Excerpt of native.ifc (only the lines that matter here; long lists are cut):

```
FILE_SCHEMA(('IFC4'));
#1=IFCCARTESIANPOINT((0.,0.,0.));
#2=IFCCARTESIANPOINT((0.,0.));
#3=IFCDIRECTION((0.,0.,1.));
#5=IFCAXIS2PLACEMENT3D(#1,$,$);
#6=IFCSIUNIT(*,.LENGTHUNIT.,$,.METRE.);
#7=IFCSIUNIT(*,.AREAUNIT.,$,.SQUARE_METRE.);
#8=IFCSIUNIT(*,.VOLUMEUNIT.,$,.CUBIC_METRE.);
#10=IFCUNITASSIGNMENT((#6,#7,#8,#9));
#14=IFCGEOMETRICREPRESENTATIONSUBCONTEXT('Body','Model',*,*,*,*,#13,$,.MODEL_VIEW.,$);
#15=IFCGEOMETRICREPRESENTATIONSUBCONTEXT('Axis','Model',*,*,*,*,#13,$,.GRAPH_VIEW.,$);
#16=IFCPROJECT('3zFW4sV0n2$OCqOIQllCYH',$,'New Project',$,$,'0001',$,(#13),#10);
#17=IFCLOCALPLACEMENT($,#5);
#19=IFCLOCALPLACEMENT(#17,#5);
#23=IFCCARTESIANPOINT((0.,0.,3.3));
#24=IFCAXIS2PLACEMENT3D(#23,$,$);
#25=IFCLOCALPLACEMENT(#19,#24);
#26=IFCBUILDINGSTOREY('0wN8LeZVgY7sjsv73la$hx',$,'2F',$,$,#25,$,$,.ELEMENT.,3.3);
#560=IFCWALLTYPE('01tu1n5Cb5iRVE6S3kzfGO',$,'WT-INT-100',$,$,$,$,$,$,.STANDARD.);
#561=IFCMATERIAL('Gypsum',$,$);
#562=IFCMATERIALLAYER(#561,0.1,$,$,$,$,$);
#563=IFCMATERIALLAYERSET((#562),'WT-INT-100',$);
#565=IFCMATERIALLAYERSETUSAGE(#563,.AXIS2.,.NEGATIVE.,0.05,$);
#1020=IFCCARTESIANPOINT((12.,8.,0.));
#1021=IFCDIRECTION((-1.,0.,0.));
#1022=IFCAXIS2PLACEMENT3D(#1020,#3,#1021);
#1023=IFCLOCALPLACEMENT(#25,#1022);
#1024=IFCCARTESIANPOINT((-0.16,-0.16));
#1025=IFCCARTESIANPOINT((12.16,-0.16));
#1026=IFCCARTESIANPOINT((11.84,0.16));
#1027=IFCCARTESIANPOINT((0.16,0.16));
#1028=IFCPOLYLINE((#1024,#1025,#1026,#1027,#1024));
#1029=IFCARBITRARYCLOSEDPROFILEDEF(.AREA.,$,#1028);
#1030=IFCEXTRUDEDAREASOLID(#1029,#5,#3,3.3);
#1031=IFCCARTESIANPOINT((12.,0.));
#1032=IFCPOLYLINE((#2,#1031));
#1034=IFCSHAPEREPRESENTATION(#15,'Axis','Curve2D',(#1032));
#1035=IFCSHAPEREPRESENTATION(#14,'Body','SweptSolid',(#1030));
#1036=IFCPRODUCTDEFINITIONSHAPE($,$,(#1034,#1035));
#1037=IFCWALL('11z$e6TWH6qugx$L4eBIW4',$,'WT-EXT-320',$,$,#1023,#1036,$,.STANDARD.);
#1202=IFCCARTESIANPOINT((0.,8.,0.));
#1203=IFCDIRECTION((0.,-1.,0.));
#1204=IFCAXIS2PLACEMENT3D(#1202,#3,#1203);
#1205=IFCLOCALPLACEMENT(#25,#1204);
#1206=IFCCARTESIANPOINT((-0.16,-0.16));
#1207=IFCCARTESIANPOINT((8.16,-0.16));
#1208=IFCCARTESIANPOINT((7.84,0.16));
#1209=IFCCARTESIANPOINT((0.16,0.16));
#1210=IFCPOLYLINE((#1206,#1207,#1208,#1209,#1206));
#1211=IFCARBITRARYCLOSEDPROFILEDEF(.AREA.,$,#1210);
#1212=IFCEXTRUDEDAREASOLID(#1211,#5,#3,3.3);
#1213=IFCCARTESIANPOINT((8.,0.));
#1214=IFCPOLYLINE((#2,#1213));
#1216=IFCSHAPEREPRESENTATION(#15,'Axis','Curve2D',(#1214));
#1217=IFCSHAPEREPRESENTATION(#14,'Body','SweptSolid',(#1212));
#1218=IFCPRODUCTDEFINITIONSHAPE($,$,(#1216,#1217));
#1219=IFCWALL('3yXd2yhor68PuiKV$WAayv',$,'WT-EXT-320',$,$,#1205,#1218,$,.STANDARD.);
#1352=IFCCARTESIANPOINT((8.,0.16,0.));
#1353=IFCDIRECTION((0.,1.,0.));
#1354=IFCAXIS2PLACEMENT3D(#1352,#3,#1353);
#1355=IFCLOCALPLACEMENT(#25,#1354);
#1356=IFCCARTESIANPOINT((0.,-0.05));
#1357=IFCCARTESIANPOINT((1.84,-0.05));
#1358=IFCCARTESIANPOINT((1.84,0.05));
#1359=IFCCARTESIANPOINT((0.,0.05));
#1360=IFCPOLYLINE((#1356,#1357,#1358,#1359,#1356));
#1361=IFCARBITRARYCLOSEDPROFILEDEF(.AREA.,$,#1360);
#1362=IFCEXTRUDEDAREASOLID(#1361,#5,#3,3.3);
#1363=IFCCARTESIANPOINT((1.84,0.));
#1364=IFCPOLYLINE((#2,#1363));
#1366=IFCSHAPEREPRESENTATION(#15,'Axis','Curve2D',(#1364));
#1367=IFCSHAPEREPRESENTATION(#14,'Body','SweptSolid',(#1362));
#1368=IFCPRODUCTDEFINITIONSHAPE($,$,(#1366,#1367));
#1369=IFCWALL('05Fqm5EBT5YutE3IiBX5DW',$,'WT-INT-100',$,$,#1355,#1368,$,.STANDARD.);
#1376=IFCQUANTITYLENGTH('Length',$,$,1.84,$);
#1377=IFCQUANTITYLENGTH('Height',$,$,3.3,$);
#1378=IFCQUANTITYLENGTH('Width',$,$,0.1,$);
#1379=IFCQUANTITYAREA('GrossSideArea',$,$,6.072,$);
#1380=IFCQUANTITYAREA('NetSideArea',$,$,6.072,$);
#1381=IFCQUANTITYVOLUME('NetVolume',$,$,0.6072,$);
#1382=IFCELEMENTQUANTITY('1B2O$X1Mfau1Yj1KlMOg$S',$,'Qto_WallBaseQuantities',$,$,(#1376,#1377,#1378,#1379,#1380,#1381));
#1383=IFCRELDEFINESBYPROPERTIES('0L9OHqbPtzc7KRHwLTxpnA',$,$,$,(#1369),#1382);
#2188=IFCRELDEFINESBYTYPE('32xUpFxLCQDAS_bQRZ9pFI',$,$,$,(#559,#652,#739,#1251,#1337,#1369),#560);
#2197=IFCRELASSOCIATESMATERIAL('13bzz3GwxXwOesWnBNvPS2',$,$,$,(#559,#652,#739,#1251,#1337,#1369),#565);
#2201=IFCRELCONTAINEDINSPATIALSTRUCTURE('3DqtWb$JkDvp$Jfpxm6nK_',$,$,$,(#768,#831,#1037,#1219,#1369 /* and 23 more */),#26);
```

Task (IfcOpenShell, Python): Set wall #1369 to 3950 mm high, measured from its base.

```python
import ifcopenshell
import ifcopenshell.api.pset
import ifcopenshell.geom
import ifcopenshell.util.element
import ifcopenshell.util.representation
import ifcopenshell.util.shape
import ifcopenshell.util.unit

model = ifcopenshell.open("native.ifc")
unit_scale = ifcopenshell.util.unit.calculate_unit_scale(model)
area_scale = ifcopenshell.util.unit.calculate_unit_scale(model, "AREAUNIT")
volume_scale = ifcopenshell.util.unit.calculate_unit_scale(model, "VOLUMEUNIT")
settings = ifcopenshell.geom.settings()


def volume(element):
    """Net volume in cubic metres, openings subtracted."""
    shape = ifcopenshell.geom.create_shape(settings, element)
    return ifcopenshell.util.shape.get_volume(shape.geometry)


wall = model.by_guid("05Fqm5EBT5YutE3IiBX5DW")
before = volume(wall)

body = ifcopenshell.util.representation.get_representation(wall, "Model", "Body")
solid = body.Items[0]
old_height = solid.Depth
solid.Depth = 3.95 / unit_scale
after = volume(wall)
thickness = 0.1  # wall thickness in metres

# Update the stored height, areas and volumes.
qto = model.by_id(ifcopenshell.util.element.get_pset(wall, "Qto_WallBaseQuantities", should_inherit=False)["id"])
ifcopenshell.api.pset.edit_qto(model, qto=qto, properties={
    "Height": solid.Depth,
    "GrossSideArea": ifcopenshell.util.element.get_pset(wall, "Qto_WallBaseQuantities", "GrossSideArea") * solid.Depth / old_height,
    "NetSideArea": after / thickness / area_scale,
    "NetVolume": after / volume_scale,
})

print(f"height {old_height:g} -> {solid.Depth:g}, volume {before:.3f} -> {after:.3f} m3")

model.write("native_edited.ifc")
```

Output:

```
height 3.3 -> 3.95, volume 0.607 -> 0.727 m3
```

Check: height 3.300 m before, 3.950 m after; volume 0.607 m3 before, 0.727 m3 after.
